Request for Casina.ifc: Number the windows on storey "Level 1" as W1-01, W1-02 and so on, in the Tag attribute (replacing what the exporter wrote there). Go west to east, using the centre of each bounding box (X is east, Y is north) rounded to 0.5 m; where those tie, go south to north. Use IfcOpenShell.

First a look at what the model holds.

```python
import ifcopenshell
import ifcopenshell.util.element
import ifcopenshell.util.placement

model = ifcopenshell.open("Casina.ifc")
print(model.schema)
storey = next(s for s in model.by_type("IfcBuildingStorey") if s.Name == "Level 1")
windows = [e for e in ifcopenshell.util.element.get_decomposition(storey) if e.is_a("IfcWindow")]
for e in sorted(windows, key=lambda e: e.id()):
    origin = ifcopenshell.util.placement.get_local_placement(e.ObjectPlacement)[:3, 3]
    print(e.id(), e.Tag, e.Name, origin.round(2) + 0.0, sep=" | ")
```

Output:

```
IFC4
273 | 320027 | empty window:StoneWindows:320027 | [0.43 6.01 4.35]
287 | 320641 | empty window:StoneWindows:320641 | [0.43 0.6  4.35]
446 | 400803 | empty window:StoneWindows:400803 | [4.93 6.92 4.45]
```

```python
import ifcopenshell
import ifcopenshell.geom
import ifcopenshell.util.element
import ifcopenshell.util.shape

model = ifcopenshell.open("Casina.ifc")
settings = ifcopenshell.geom.settings()
settings.set("use-world-coords", True)


def centre(element):
    shape = ifcopenshell.geom.create_shape(settings, element)
    return ifcopenshell.util.shape.get_bbox_centroid(shape.geometry)


storey = next(s for s in model.by_type("IfcBuildingStorey") if s.Name == "Level 1")
windows = [e for e in ifcopenshell.util.element.get_decomposition(storey) if e.is_a("IfcWindow")]

# Insertion points can sit at a corner or the storey origin, so sort by the geometry (in metres).
centres = {e: centre(e) for e in windows}
windows.sort(key=lambda e: (round(centres[e][0] / 0.5), centres[e][1]))

for i, e in enumerate(windows, start=1):
    number = f"W1-{i:02d}"
    e.Tag = number
    print(e.id(), number)

model.write("Casina_edited.ifc")
```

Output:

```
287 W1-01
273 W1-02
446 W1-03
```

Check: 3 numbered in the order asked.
